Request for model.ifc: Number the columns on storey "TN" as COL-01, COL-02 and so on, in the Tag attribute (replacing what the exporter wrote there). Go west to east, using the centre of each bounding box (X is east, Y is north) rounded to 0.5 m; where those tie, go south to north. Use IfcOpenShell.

First a look at what the model holds.

```python
import ifcopenshell
import ifcopenshell.util.element
import ifcopenshell.util.placement

model = ifcopenshell.open("model.ifc")
print(model.schema)
storey = next(s for s in model.by_type("IfcBuildingStorey") if s.Name == "TN")
columns = [e for e in ifcopenshell.util.element.get_decomposition(storey) if e.is_a("IfcColumn")]
for e in sorted(columns, key=lambda e: e.id()):
    origin = ifcopenshell.util.placement.get_local_placement(e.ObjectPlacement)[:3, 3]
    print(e.id(), e.Tag, e.Name, origin.round(2) + 0.0, sep=" | ")
```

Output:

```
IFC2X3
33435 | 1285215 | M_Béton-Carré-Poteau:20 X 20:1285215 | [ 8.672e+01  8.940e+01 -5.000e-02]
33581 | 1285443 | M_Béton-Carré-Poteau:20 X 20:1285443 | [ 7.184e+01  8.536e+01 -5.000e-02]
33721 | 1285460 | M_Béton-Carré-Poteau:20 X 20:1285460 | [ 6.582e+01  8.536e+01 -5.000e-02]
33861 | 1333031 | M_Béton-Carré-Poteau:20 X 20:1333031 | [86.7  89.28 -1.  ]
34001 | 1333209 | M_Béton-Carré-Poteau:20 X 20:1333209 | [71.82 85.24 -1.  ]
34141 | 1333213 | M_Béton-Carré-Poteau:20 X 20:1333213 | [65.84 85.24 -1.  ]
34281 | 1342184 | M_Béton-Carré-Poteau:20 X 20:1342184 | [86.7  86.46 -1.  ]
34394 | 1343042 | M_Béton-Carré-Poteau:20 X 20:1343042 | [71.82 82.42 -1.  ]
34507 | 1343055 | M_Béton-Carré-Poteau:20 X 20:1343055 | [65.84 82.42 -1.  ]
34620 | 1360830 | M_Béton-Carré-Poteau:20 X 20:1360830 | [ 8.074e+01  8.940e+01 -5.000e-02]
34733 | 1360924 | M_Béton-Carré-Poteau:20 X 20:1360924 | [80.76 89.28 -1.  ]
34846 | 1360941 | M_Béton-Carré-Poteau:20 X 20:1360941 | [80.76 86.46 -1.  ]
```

```python
import ifcopenshell
import ifcopenshell.geom
import ifcopenshell.util.element
import ifcopenshell.util.shape

model = ifcopenshell.open("model.ifc")
settings = ifcopenshell.geom.settings()
settings.set("use-world-coords", True)


def centre(element):
    shape = ifcopenshell.geom.create_shape(settings, element)
    return ifcopenshell.util.shape.get_bbox_centroid(shape.geometry)


storey = next(s for s in model.by_type("IfcBuildingStorey") if s.Name == "TN")
columns = [e for e in ifcopenshell.util.element.get_decomposition(storey) if e.is_a("IfcColumn")]

# Insertion points can sit at a corner or the storey origin, so sort by the geometry (in metres).
centres = {e: centre(e) for e in columns}
columns.sort(key=lambda e: (round(centres[e][0] / 0.5), centres[e][1]))

for i, e in enumerate(columns, start=1):
    number = f"COL-{i:02d}"
    e.Tag = number
    print(e.id(), number)

model.write("model_v2.ifc")
```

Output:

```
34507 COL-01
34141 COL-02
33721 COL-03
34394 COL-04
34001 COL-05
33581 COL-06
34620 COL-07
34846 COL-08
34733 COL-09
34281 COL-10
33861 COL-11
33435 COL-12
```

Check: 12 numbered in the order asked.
